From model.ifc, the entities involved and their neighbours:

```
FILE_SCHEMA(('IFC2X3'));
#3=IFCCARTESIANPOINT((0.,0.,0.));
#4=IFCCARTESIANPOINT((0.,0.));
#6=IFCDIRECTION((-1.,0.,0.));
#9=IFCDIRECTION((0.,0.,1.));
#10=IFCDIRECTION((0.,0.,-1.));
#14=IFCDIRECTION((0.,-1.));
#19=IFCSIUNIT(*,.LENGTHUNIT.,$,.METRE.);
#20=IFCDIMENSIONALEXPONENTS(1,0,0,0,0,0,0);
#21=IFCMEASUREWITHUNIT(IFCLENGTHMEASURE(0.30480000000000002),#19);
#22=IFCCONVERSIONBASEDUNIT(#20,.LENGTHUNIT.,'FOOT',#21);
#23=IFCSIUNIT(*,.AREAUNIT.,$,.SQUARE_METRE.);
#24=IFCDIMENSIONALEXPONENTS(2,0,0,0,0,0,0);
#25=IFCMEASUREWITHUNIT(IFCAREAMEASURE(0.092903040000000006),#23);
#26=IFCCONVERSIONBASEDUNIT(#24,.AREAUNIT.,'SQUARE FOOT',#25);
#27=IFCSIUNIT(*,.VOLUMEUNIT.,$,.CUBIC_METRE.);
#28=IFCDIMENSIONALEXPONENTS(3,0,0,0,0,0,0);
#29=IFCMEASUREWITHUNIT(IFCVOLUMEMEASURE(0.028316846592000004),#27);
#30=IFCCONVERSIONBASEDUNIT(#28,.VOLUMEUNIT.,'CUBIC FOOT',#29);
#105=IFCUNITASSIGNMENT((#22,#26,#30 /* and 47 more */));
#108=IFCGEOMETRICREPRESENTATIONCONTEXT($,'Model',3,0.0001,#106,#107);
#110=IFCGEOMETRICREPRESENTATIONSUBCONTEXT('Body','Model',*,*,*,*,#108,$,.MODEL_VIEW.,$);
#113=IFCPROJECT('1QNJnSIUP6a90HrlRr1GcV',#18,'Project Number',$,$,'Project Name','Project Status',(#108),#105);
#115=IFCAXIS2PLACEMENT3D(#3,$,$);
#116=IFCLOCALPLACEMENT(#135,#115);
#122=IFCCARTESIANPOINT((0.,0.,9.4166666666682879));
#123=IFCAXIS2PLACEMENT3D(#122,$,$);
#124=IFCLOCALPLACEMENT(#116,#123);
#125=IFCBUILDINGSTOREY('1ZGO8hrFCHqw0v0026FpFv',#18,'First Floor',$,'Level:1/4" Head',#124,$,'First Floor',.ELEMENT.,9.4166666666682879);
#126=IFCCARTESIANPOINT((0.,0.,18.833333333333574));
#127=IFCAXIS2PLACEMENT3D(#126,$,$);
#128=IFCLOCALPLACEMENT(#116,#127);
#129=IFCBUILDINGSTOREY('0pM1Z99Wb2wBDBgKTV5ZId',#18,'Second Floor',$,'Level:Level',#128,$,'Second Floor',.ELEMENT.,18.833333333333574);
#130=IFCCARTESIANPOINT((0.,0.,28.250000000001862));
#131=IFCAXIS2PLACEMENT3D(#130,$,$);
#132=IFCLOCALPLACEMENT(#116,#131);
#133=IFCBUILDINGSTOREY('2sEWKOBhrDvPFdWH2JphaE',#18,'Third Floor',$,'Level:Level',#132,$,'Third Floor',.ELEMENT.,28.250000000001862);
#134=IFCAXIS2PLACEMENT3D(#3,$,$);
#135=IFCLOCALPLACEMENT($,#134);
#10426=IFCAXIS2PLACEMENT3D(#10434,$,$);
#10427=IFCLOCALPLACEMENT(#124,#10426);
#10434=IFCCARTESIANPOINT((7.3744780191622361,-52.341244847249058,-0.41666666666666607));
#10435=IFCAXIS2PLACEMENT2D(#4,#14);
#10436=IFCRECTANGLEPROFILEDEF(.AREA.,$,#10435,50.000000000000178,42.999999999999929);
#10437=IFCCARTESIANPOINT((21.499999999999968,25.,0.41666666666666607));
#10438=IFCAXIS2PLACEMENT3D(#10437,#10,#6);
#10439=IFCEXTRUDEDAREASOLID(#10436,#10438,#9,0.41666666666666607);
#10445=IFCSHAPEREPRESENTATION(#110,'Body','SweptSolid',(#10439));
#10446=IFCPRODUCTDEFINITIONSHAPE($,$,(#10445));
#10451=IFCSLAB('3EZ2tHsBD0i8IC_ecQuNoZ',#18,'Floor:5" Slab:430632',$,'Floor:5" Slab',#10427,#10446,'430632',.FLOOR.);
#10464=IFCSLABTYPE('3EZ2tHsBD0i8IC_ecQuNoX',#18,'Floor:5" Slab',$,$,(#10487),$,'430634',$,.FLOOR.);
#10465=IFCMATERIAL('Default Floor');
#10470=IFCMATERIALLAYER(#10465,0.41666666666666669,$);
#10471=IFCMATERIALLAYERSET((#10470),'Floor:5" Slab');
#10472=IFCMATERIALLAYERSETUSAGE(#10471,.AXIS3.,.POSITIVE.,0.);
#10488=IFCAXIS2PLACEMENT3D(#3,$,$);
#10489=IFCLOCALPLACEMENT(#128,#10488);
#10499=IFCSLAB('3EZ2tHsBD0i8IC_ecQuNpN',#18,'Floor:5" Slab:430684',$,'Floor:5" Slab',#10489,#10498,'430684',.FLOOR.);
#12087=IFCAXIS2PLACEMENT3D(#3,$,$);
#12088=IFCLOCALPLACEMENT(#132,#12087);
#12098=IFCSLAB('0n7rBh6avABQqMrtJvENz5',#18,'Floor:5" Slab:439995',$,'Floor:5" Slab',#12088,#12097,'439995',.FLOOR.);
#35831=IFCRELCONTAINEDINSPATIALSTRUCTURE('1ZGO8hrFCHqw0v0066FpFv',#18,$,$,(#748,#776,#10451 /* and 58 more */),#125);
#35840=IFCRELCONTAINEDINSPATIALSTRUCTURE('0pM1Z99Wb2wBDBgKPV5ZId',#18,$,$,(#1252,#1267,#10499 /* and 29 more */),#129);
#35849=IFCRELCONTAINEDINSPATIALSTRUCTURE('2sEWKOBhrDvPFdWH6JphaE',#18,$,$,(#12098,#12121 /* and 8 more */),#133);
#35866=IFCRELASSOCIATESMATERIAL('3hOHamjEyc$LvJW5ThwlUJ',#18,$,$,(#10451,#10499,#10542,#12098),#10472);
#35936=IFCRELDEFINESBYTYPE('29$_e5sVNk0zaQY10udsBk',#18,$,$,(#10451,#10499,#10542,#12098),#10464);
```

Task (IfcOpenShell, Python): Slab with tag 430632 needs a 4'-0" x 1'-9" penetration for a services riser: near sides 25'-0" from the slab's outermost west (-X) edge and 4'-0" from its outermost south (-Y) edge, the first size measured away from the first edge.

```python
import numpy as np
import ifcopenshell
import ifcopenshell.api.feature
import ifcopenshell.api.geometry
import ifcopenshell.api.root
import ifcopenshell.geom
import ifcopenshell.util.placement
import ifcopenshell.util.representation
import ifcopenshell.util.shape
import ifcopenshell.util.unit

model = ifcopenshell.open("model.ifc")
unit_scale = ifcopenshell.util.unit.calculate_unit_scale(model)
settings = ifcopenshell.geom.settings()


def volume(element):
    """Net volume in cubic metres, openings subtracted."""
    shape = ifcopenshell.geom.create_shape(settings, element)
    return ifcopenshell.util.shape.get_volume(shape.geometry)


slab = model.by_id(10451)
before = volume(slab)

# Extent in the slab's own axes, in metres. The edges named are its -X and -Y sides.
slab_shape = ifcopenshell.geom.create_shape(settings, slab)
vertices = ifcopenshell.util.shape.get_vertices(slab_shape.geometry)
x_min, y_min, bottom = vertices.min(axis=0)
top = vertices[:, 2].max()

opening = ifcopenshell.api.root.create_entity(model, ifc_class="IfcOpeningElement", name="Services riser opening")
context = ifcopenshell.util.representation.get_context(model, "Model", "Body", "MODEL_VIEW")
width, depth = 1.2192, 0.5334
outline = [(0.0, 0.0), (width, 0.0), (width, depth), (0.0, depth), (0.0, 0.0)]
# Overshoot both faces by 50 mm so the cut is clean.
shape = ifcopenshell.api.geometry.add_slab_representation(
    model, context=context, depth=top - bottom + 0.1, polyline=outline
)
ifcopenshell.api.geometry.assign_representation(model, product=opening, representation=shape)

matrix = ifcopenshell.util.placement.get_local_placement(slab.ObjectPlacement)
matrix[:, 3] = matrix @ np.append(np.array([x_min + 7.62, y_min + 1.2192, bottom - 0.05]) / unit_scale, 1.0)
ifcopenshell.api.geometry.edit_object_placement(model, product=opening, matrix=matrix, is_si=False)
ifcopenshell.api.feature.add_feature(model, feature=opening, element=slab)

after = volume(slab)

print(f"slab volume {before:.3f} -> {after:.3f} m3")

model.write("model_edited.ifc")
```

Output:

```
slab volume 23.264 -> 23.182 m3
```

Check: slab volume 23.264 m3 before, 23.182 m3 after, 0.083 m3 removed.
